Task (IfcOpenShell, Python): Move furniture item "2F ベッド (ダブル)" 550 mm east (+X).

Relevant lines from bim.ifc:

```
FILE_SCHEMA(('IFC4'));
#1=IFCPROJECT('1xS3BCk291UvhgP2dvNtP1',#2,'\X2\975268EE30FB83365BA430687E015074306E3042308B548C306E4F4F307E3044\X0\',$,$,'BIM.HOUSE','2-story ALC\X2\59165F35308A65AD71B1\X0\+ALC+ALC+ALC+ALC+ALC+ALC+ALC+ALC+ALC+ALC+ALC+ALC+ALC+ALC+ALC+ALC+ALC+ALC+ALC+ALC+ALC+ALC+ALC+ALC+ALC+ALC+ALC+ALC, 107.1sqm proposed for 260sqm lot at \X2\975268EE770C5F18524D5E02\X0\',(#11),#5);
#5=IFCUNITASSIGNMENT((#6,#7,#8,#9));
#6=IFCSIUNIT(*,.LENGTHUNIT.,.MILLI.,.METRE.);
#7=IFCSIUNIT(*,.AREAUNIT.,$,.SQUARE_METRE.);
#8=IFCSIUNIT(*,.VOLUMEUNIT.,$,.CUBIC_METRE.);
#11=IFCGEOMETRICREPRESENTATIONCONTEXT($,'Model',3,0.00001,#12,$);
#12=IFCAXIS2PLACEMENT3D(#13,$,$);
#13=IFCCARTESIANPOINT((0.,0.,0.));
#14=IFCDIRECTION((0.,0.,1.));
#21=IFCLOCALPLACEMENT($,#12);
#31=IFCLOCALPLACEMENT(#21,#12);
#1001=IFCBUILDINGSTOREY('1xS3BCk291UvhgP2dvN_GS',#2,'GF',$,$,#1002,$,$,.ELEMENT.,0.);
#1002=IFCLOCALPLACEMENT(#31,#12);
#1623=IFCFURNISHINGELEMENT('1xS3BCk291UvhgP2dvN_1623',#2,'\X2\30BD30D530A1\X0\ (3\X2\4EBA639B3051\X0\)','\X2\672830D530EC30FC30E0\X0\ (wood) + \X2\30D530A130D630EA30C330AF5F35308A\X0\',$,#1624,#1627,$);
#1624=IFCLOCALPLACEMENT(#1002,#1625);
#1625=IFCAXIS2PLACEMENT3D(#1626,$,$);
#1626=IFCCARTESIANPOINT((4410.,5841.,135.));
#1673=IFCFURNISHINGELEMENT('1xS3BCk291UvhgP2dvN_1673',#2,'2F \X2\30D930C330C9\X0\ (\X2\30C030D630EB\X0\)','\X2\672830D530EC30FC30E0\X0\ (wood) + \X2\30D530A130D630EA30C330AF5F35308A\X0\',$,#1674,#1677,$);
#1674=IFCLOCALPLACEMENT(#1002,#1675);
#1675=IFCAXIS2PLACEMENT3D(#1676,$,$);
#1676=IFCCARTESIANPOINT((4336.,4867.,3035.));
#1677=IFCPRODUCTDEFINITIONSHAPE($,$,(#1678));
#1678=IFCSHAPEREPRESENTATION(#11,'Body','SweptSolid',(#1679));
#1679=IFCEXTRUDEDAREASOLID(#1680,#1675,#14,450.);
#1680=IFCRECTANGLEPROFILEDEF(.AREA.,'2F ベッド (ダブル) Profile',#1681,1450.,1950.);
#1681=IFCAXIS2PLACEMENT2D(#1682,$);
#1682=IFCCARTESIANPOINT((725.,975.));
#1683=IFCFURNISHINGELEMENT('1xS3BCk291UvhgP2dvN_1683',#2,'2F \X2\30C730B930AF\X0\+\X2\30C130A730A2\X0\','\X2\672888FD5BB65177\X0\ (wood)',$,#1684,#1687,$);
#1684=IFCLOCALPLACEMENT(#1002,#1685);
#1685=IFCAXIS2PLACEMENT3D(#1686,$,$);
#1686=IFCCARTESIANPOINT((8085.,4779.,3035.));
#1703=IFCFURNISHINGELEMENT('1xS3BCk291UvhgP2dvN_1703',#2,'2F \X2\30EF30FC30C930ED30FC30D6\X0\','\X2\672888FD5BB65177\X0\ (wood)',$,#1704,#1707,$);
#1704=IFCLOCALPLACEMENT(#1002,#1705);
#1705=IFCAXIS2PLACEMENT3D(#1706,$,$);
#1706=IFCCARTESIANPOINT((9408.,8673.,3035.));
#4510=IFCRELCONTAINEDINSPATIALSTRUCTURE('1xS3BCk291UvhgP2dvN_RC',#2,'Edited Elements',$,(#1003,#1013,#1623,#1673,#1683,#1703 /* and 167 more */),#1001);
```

```python
import ifcopenshell
import ifcopenshell.api.geometry
import ifcopenshell.util.placement
import ifcopenshell.util.unit

model = ifcopenshell.open("bim.ifc")
unit_scale = ifcopenshell.util.unit.calculate_unit_scale(model)

item = model.by_guid("1xS3BCk291UvhgP2dvN_1673")
matrix = ifcopenshell.util.placement.get_local_placement(item.ObjectPlacement)
matrix[0, 3] += 0.55 / unit_scale
ifcopenshell.api.geometry.edit_object_placement(model, product=item, matrix=matrix, is_si=False)

print(ifcopenshell.util.placement.get_local_placement(item.ObjectPlacement).round(3) + 0.0)

model.write("bim_v2.ifc")
```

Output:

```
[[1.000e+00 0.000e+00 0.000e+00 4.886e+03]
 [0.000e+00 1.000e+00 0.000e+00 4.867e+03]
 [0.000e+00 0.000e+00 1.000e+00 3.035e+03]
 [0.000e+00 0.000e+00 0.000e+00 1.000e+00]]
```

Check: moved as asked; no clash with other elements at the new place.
